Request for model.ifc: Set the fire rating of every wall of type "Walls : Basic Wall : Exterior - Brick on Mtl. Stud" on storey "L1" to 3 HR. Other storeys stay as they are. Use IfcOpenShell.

First a look at what the model holds.

```python
import ifcopenshell
import ifcopenshell.util.element

model = ifcopenshell.open("model.ifc")
print(model.schema)
storey = next(s for s in model.by_type("IfcBuildingStorey") if s.Name == "L1")
walls = [e for e in ifcopenshell.util.element.get_decomposition(storey) if e.is_a("IfcWall")]
seen = {}
for e in walls:
    element_type = ifcopenshell.util.element.get_type(e)
    key = (element_type.Name if element_type != e and element_type else None, ifcopenshell.util.element.get_pset(e, "Pset_WallCommon", "FireRating"))
    seen[key] = seen.get(key, 0) + 1
for (name, value), count in sorted(seen.items(), key=str):
    print(count, "x", name, "|", value)
```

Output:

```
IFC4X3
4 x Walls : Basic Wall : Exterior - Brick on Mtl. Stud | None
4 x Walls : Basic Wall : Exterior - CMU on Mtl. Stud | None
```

```python
import ifcopenshell
import ifcopenshell.api.pset
import ifcopenshell.util.element

model = ifcopenshell.open("model.ifc")

storey = next(s for s in model.by_type("IfcBuildingStorey") if s.Name == "L1")
walls = [e for e in ifcopenshell.util.element.get_decomposition(storey) if e.is_a("IfcWall")]

count = 0
for e in walls:
    element_type = ifcopenshell.util.element.get_type(e)
    if element_type in (None, e) or element_type.Name != "Walls : Basic Wall : Exterior - Brick on Mtl. Stud":
        continue
    # add_pset returns the element's existing set when there is one.
    pset = ifcopenshell.api.pset.add_pset(model, product=e, name="Pset_WallCommon")
    ifcopenshell.api.pset.edit_pset(model, pset=pset, properties={"FireRating": "3 HR"})
    count += 1

print(count, "walls updated")

model.write("model_updated.ifc")
```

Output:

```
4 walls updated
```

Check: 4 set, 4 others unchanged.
